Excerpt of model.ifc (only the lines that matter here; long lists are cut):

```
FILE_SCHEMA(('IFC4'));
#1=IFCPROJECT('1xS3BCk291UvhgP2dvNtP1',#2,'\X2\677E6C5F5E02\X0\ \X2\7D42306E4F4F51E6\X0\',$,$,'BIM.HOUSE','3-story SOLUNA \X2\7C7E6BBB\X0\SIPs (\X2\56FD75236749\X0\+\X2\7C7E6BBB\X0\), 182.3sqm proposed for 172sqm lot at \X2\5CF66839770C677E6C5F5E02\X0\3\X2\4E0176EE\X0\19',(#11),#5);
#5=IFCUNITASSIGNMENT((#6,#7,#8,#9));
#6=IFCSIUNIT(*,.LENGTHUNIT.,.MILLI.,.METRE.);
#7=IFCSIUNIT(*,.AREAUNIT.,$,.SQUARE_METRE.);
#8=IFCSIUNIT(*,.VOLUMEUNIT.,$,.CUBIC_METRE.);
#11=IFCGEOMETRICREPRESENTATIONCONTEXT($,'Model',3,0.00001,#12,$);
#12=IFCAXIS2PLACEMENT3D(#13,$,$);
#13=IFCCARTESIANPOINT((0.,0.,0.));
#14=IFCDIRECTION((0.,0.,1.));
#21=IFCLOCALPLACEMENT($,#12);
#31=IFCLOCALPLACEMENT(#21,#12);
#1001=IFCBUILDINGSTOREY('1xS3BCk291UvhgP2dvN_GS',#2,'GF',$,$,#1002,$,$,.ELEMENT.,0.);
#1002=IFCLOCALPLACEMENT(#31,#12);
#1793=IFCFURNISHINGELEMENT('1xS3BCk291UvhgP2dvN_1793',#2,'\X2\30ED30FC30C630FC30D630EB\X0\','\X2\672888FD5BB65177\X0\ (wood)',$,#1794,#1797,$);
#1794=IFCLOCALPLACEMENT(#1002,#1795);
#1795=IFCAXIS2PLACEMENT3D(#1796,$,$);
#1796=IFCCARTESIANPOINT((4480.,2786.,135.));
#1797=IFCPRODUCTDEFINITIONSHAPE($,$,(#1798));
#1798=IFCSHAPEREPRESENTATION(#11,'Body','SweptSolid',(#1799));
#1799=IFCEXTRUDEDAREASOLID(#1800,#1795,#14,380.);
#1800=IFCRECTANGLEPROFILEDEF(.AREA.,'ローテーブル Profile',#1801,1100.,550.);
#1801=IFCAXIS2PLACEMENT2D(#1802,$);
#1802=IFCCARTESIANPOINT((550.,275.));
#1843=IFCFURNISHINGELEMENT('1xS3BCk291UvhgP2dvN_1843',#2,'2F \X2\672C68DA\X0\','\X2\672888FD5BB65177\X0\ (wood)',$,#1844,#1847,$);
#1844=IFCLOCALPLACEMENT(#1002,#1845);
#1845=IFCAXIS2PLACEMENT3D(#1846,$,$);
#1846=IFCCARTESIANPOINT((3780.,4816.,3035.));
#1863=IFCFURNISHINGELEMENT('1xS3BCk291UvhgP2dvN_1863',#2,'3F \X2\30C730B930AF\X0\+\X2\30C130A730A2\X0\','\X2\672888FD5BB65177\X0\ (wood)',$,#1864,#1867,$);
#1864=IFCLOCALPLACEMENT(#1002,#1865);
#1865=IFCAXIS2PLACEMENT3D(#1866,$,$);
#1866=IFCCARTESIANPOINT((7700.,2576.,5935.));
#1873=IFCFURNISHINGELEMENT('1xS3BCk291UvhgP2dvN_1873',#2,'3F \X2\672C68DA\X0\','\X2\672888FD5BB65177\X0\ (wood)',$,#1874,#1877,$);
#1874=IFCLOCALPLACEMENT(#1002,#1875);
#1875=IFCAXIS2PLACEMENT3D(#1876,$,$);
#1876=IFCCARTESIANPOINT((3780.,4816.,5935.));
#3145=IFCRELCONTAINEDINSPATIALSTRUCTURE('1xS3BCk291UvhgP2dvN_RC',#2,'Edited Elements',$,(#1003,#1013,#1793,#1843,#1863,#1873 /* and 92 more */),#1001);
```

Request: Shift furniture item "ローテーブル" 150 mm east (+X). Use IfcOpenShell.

```python
import ifcopenshell
import ifcopenshell.api.geometry
import ifcopenshell.util.placement

model = ifcopenshell.open("model.ifc")

item = model.by_id(1793)
matrix = ifcopenshell.util.placement.get_local_placement(item.ObjectPlacement)
matrix[0, 3] += 150.0
ifcopenshell.api.geometry.edit_object_placement(model, product=item, matrix=matrix, is_si=False)

print(ifcopenshell.util.placement.get_local_placement(item.ObjectPlacement).round(3) + 0.0)

model.write("model_updated.ifc")
```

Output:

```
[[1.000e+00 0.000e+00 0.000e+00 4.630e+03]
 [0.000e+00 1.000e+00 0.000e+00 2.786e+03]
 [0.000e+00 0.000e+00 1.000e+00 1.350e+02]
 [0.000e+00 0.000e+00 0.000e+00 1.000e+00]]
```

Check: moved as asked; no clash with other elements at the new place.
